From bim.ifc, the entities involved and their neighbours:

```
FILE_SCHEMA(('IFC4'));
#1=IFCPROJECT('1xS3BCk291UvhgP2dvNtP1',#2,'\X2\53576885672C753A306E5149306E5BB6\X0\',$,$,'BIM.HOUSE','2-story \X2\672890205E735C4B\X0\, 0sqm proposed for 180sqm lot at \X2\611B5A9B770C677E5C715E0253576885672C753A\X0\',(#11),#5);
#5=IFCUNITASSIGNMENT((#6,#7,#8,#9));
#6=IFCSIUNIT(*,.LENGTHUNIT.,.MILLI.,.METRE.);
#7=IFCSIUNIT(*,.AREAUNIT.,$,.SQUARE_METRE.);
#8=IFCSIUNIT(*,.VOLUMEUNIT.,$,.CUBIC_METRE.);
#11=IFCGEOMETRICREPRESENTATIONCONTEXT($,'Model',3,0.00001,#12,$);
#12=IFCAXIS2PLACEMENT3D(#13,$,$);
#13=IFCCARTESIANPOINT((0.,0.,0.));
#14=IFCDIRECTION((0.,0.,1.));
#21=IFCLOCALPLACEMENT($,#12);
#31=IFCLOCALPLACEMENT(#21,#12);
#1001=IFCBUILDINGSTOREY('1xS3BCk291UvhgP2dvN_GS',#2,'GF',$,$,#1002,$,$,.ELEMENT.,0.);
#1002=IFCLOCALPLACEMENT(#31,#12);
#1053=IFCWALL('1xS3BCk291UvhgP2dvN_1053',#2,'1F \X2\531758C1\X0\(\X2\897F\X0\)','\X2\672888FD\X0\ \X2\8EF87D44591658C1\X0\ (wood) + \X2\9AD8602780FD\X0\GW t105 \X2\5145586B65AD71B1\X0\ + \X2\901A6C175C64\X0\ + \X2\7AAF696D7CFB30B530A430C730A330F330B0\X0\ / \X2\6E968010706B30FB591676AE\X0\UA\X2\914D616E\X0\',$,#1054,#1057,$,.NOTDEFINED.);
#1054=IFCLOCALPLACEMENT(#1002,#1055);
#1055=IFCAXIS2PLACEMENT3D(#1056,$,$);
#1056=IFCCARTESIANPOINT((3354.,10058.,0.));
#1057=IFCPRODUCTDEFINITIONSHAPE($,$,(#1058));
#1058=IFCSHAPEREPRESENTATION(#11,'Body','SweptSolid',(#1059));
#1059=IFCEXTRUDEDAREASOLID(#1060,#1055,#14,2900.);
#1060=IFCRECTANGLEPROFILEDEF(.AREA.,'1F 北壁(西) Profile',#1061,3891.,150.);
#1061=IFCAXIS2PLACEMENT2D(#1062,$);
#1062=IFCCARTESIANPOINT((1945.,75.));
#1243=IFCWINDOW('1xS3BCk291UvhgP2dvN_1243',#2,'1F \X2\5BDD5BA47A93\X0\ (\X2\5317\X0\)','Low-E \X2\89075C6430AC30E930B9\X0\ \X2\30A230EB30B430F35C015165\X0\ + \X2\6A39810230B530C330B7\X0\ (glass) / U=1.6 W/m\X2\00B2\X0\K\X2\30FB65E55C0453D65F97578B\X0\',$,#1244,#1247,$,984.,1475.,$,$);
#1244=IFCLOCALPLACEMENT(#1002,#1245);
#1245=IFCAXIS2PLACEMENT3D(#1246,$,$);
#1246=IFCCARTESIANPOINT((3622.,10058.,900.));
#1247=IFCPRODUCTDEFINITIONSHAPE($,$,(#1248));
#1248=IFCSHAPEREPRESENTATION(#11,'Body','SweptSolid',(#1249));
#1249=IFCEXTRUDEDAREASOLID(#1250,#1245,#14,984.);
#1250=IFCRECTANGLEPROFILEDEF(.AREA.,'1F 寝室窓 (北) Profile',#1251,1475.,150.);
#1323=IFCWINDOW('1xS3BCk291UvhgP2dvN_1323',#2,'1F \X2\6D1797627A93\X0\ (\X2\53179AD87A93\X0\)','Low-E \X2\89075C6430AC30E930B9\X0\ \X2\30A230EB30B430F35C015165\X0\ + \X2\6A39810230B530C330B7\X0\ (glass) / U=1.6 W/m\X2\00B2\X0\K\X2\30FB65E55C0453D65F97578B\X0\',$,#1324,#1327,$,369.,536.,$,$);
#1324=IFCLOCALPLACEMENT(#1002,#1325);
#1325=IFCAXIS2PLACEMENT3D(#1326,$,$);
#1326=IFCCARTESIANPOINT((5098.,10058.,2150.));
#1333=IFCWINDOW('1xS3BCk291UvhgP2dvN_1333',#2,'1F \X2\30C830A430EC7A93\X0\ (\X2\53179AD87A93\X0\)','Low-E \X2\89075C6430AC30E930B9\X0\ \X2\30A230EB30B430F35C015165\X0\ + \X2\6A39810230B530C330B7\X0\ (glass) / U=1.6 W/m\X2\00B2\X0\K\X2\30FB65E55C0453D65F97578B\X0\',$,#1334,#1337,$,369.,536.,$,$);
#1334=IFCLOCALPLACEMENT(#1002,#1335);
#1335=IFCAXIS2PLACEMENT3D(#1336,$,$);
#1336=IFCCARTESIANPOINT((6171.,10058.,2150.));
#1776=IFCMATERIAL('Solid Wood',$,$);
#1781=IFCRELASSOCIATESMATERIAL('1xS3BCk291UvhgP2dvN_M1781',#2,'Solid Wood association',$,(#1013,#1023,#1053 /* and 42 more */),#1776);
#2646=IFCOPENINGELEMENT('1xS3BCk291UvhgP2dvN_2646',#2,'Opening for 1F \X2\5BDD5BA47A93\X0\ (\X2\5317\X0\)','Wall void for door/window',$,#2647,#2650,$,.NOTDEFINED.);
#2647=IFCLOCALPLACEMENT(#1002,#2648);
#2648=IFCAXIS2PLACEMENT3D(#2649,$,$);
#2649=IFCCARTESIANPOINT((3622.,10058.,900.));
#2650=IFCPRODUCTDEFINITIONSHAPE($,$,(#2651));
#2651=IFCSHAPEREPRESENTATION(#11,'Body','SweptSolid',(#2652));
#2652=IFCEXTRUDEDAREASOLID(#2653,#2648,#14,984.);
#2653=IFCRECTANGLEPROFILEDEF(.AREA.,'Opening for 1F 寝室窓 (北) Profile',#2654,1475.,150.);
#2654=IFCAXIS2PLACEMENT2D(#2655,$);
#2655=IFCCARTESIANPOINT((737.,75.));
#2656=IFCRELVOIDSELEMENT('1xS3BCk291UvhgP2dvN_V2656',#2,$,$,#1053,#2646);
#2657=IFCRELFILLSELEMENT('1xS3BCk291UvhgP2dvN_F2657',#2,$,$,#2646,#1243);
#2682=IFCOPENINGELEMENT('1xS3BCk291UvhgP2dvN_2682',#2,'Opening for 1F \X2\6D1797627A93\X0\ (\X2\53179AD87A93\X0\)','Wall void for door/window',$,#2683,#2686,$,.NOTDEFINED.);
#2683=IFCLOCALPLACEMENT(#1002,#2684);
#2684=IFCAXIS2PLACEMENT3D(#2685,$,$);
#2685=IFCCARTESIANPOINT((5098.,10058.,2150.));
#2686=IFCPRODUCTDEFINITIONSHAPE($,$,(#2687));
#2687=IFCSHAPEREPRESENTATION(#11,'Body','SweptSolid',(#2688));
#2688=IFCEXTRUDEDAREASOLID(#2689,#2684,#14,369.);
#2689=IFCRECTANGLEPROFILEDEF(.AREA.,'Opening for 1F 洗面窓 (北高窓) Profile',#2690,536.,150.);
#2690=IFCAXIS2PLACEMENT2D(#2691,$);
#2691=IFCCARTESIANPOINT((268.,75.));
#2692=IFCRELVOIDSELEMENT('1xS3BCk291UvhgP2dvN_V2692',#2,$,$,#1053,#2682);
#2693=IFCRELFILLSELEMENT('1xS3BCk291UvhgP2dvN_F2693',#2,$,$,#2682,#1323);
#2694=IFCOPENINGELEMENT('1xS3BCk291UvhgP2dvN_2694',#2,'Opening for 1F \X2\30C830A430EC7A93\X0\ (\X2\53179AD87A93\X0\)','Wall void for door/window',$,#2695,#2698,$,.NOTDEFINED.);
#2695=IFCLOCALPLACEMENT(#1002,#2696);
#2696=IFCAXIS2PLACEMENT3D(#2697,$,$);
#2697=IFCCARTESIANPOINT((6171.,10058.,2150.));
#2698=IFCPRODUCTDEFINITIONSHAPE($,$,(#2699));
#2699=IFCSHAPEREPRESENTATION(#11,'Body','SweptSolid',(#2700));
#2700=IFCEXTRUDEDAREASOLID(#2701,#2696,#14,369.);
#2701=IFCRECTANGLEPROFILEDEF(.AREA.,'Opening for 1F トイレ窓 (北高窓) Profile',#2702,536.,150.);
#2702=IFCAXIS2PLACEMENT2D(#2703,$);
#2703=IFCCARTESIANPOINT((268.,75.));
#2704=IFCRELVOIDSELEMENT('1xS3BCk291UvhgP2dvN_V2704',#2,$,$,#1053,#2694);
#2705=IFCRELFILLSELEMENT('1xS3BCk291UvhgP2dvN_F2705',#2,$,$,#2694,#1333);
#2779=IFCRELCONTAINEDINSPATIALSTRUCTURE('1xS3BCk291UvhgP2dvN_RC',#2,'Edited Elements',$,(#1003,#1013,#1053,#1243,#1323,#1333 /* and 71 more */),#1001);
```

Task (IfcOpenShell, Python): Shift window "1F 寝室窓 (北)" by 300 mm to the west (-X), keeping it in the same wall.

```python
import ifcopenshell
import ifcopenshell.api.geometry
import ifcopenshell.util.placement
import ifcopenshell.util.unit

model = ifcopenshell.open("bim.ifc")
unit_scale = ifcopenshell.util.unit.calculate_unit_scale(model)

window = model.by_id(1243)
opening = window.FillsVoids[0].RelatingOpeningElement
wall = opening.VoidsElements[0].RelatingBuildingElement

wall_matrix = ifcopenshell.util.placement.get_local_placement(wall.ObjectPlacement)
shift = wall_matrix[:3, 0] * -0.3 / unit_scale
before = ifcopenshell.util.placement.get_local_placement(window.ObjectPlacement)[:3, 3].copy()

# The window is not placed relative to its opening, so move both.
for product in (opening, window):
    matrix = ifcopenshell.util.placement.get_local_placement(product.ObjectPlacement)
    matrix[:3, 3] += shift
    ifcopenshell.api.geometry.edit_object_placement(model, product=product, matrix=matrix, is_si=False)

after = ifcopenshell.util.placement.get_local_placement(window.ObjectPlacement)[:3, 3]
print("window moved by", (after - before).round(3) + 0.0)

model.write("bim_rev.ifc")
```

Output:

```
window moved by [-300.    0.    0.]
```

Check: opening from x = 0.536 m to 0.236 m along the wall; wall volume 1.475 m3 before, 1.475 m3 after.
